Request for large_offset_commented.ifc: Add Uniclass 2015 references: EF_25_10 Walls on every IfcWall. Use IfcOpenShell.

First a look at what the model holds.

```python
import ifcopenshell

model = ifcopenshell.open("large_offset_commented.ifc")
print(model.schema)
print("classifications:", [c.Name for c in model.by_type("IfcClassification")])
for ifc_class in ("IfcDoor", "IfcRoof", "IfcStair", "IfcWall", "IfcWindow"):
    print(ifc_class, len(model.by_type(ifc_class)))
```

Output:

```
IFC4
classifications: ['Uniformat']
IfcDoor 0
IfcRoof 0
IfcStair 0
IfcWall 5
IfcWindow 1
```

```python
import ifcopenshell
import ifcopenshell.api.classification

model = ifcopenshell.open("large_offset_commented.ifc")

system = ifcopenshell.api.classification.add_classification(model, classification="Uniclass 2015")

codes = {
    "IfcWall": ("EF_25_10", "Walls"),
}
for ifc_class, (code, name) in codes.items():
    products = model.by_type(ifc_class)
    ifcopenshell.api.classification.add_reference(
        model, products=products, classification=system, identification=code, name=name
    )
    print(code, len(products))

model.write("large_offset_commented_edited.ifc")
```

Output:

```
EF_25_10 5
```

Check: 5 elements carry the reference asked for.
